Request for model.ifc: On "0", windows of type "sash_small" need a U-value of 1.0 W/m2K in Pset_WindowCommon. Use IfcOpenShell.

First a look at what the model holds.

```python
import ifcopenshell
import ifcopenshell.util.element

model = ifcopenshell.open("model.ifc")
print(model.schema)
storey = next(s for s in model.by_type("IfcBuildingStorey") if s.Name == "0")
windows = [e for e in ifcopenshell.util.element.get_decomposition(storey) if e.is_a("IfcWindow")]
seen = {}
for e in windows:
    element_type = ifcopenshell.util.element.get_type(e)
    key = (element_type.Name if element_type != e and element_type else None, ifcopenshell.util.element.get_pset(e, "Pset_WindowCommon", "ThermalTransmittance"))
    seen[key] = seen.get(key, 0) + 1
for (name, value), count in sorted(seen.items(), key=str):
    print(count, "x", name, "|", value)
```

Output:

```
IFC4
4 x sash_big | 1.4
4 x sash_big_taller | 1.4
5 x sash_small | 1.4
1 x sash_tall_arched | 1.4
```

```python
import ifcopenshell
import ifcopenshell.api.pset
import ifcopenshell.util.element

model = ifcopenshell.open("model.ifc")

storey = next(s for s in model.by_type("IfcBuildingStorey") if s.Name == "0")
windows = [e for e in ifcopenshell.util.element.get_decomposition(storey) if e.is_a("IfcWindow")]

count = 0
for e in windows:
    element_type = ifcopenshell.util.element.get_type(e)
    if element_type in (None, e) or element_type.Name != "sash_small":
        continue
    # add_pset returns the element's existing set when there is one.
    pset = ifcopenshell.api.pset.add_pset(model, product=e, name="Pset_WindowCommon")
    ifcopenshell.api.pset.edit_pset(model, pset=pset, properties={"ThermalTransmittance": 1.0})
    count += 1

print(count, "windows updated")

model.write("model_updated.ifc")
```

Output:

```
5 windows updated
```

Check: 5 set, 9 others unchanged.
